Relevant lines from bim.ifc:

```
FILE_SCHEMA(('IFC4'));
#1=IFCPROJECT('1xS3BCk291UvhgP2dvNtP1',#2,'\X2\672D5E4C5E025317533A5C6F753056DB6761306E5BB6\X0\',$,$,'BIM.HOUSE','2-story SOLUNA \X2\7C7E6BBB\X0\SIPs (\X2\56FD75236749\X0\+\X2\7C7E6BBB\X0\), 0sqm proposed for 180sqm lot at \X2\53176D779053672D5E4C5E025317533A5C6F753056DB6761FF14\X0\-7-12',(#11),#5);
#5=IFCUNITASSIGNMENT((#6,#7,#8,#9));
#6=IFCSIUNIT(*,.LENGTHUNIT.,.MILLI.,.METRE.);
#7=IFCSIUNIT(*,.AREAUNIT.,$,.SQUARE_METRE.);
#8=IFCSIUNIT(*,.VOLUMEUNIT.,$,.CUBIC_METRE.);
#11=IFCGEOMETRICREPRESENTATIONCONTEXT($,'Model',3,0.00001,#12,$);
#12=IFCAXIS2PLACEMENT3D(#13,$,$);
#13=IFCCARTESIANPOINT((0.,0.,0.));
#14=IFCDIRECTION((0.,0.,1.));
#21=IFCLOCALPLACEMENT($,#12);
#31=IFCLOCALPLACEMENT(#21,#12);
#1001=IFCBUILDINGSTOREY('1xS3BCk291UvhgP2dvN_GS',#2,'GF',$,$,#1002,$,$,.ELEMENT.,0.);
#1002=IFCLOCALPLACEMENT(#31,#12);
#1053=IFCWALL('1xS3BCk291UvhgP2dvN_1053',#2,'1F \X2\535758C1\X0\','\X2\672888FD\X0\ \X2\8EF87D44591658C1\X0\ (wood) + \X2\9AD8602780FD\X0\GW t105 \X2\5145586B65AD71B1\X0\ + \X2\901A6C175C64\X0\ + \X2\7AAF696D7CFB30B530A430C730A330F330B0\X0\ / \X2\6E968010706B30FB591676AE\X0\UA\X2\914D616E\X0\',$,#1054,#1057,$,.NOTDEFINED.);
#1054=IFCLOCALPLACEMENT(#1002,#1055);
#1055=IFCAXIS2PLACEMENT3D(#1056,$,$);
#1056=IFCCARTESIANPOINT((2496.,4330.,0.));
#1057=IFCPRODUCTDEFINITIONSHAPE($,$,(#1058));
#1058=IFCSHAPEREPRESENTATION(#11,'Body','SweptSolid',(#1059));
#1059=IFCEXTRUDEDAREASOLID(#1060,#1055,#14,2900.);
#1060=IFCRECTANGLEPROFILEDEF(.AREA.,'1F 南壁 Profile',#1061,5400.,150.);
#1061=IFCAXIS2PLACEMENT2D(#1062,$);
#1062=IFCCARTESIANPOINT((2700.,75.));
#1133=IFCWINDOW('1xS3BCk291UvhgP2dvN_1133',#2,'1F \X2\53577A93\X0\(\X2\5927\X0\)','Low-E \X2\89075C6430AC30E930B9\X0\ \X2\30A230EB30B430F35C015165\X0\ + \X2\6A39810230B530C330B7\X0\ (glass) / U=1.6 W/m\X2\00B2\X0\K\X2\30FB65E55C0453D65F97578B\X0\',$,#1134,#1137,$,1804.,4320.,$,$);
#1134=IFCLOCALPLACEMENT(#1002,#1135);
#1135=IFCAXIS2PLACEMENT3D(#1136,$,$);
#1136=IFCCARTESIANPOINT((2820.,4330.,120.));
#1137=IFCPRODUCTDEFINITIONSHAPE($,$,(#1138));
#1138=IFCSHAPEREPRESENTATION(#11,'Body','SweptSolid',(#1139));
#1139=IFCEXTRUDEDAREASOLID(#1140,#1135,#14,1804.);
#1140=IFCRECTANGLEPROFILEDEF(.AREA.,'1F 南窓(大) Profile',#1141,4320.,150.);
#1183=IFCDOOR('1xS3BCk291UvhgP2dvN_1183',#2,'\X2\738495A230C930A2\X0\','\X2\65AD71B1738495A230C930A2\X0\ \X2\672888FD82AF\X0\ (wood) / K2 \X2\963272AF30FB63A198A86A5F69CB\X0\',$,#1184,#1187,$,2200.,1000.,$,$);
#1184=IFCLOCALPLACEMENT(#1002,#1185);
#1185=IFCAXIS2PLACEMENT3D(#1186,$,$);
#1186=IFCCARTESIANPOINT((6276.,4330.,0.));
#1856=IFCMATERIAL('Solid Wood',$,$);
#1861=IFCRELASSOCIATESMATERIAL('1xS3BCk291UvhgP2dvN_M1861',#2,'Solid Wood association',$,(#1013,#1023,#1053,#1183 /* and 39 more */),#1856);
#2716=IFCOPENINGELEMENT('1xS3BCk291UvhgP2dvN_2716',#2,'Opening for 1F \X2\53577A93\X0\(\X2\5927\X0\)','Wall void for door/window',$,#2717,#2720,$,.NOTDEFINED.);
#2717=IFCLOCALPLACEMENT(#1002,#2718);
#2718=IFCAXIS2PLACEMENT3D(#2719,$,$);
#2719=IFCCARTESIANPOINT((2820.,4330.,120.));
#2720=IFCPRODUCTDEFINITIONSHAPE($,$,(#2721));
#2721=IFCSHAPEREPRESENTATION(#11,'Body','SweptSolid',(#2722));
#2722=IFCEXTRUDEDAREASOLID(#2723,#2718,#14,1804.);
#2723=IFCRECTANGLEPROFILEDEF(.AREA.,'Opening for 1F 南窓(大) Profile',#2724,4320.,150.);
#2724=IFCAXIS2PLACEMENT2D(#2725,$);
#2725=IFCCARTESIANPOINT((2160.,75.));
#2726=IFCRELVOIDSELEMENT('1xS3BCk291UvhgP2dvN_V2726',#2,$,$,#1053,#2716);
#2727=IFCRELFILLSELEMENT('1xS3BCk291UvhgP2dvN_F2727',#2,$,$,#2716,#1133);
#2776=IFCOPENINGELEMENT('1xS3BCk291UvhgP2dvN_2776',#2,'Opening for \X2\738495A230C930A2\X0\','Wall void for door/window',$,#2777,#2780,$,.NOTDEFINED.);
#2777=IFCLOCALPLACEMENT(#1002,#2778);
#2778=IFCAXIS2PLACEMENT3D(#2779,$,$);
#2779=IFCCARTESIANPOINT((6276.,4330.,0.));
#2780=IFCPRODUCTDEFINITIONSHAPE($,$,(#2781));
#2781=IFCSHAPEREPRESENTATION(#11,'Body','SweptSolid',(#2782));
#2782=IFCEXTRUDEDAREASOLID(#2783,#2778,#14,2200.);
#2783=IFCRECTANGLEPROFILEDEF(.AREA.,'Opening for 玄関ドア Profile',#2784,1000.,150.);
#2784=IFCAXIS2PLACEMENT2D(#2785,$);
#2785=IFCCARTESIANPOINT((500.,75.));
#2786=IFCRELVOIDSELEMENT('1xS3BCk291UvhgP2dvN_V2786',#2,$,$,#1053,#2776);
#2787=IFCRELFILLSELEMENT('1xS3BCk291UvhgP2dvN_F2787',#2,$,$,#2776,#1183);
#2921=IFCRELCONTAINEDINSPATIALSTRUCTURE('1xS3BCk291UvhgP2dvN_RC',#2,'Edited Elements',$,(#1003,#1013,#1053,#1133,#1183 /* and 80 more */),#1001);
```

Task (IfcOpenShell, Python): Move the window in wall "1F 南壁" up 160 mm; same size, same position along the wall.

```python
import numpy as np
import ifcopenshell
import ifcopenshell.api.geometry
import ifcopenshell.util.placement
import ifcopenshell.util.unit

model = ifcopenshell.open("bim.ifc")
unit_scale = ifcopenshell.util.unit.calculate_unit_scale(model)

window = model.by_guid("1xS3BCk291UvhgP2dvN_1133")
opening = window.FillsVoids[0].RelatingOpeningElement
dz = 0.16 / unit_scale

shift = np.array([0.0, 0.0, dz])
# The window is not placed relative to its opening, so move both.
for product in (opening, window):
    matrix = ifcopenshell.util.placement.get_local_placement(product.ObjectPlacement)
    matrix[:3, 3] += shift
    ifcopenshell.api.geometry.edit_object_placement(model, product=product, matrix=matrix, is_si=False)

print(f"moved by {dz * unit_scale:+.3f} m")

model.write("bim_edited.ifc")
```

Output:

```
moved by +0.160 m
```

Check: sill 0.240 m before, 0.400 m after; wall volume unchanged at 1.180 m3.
